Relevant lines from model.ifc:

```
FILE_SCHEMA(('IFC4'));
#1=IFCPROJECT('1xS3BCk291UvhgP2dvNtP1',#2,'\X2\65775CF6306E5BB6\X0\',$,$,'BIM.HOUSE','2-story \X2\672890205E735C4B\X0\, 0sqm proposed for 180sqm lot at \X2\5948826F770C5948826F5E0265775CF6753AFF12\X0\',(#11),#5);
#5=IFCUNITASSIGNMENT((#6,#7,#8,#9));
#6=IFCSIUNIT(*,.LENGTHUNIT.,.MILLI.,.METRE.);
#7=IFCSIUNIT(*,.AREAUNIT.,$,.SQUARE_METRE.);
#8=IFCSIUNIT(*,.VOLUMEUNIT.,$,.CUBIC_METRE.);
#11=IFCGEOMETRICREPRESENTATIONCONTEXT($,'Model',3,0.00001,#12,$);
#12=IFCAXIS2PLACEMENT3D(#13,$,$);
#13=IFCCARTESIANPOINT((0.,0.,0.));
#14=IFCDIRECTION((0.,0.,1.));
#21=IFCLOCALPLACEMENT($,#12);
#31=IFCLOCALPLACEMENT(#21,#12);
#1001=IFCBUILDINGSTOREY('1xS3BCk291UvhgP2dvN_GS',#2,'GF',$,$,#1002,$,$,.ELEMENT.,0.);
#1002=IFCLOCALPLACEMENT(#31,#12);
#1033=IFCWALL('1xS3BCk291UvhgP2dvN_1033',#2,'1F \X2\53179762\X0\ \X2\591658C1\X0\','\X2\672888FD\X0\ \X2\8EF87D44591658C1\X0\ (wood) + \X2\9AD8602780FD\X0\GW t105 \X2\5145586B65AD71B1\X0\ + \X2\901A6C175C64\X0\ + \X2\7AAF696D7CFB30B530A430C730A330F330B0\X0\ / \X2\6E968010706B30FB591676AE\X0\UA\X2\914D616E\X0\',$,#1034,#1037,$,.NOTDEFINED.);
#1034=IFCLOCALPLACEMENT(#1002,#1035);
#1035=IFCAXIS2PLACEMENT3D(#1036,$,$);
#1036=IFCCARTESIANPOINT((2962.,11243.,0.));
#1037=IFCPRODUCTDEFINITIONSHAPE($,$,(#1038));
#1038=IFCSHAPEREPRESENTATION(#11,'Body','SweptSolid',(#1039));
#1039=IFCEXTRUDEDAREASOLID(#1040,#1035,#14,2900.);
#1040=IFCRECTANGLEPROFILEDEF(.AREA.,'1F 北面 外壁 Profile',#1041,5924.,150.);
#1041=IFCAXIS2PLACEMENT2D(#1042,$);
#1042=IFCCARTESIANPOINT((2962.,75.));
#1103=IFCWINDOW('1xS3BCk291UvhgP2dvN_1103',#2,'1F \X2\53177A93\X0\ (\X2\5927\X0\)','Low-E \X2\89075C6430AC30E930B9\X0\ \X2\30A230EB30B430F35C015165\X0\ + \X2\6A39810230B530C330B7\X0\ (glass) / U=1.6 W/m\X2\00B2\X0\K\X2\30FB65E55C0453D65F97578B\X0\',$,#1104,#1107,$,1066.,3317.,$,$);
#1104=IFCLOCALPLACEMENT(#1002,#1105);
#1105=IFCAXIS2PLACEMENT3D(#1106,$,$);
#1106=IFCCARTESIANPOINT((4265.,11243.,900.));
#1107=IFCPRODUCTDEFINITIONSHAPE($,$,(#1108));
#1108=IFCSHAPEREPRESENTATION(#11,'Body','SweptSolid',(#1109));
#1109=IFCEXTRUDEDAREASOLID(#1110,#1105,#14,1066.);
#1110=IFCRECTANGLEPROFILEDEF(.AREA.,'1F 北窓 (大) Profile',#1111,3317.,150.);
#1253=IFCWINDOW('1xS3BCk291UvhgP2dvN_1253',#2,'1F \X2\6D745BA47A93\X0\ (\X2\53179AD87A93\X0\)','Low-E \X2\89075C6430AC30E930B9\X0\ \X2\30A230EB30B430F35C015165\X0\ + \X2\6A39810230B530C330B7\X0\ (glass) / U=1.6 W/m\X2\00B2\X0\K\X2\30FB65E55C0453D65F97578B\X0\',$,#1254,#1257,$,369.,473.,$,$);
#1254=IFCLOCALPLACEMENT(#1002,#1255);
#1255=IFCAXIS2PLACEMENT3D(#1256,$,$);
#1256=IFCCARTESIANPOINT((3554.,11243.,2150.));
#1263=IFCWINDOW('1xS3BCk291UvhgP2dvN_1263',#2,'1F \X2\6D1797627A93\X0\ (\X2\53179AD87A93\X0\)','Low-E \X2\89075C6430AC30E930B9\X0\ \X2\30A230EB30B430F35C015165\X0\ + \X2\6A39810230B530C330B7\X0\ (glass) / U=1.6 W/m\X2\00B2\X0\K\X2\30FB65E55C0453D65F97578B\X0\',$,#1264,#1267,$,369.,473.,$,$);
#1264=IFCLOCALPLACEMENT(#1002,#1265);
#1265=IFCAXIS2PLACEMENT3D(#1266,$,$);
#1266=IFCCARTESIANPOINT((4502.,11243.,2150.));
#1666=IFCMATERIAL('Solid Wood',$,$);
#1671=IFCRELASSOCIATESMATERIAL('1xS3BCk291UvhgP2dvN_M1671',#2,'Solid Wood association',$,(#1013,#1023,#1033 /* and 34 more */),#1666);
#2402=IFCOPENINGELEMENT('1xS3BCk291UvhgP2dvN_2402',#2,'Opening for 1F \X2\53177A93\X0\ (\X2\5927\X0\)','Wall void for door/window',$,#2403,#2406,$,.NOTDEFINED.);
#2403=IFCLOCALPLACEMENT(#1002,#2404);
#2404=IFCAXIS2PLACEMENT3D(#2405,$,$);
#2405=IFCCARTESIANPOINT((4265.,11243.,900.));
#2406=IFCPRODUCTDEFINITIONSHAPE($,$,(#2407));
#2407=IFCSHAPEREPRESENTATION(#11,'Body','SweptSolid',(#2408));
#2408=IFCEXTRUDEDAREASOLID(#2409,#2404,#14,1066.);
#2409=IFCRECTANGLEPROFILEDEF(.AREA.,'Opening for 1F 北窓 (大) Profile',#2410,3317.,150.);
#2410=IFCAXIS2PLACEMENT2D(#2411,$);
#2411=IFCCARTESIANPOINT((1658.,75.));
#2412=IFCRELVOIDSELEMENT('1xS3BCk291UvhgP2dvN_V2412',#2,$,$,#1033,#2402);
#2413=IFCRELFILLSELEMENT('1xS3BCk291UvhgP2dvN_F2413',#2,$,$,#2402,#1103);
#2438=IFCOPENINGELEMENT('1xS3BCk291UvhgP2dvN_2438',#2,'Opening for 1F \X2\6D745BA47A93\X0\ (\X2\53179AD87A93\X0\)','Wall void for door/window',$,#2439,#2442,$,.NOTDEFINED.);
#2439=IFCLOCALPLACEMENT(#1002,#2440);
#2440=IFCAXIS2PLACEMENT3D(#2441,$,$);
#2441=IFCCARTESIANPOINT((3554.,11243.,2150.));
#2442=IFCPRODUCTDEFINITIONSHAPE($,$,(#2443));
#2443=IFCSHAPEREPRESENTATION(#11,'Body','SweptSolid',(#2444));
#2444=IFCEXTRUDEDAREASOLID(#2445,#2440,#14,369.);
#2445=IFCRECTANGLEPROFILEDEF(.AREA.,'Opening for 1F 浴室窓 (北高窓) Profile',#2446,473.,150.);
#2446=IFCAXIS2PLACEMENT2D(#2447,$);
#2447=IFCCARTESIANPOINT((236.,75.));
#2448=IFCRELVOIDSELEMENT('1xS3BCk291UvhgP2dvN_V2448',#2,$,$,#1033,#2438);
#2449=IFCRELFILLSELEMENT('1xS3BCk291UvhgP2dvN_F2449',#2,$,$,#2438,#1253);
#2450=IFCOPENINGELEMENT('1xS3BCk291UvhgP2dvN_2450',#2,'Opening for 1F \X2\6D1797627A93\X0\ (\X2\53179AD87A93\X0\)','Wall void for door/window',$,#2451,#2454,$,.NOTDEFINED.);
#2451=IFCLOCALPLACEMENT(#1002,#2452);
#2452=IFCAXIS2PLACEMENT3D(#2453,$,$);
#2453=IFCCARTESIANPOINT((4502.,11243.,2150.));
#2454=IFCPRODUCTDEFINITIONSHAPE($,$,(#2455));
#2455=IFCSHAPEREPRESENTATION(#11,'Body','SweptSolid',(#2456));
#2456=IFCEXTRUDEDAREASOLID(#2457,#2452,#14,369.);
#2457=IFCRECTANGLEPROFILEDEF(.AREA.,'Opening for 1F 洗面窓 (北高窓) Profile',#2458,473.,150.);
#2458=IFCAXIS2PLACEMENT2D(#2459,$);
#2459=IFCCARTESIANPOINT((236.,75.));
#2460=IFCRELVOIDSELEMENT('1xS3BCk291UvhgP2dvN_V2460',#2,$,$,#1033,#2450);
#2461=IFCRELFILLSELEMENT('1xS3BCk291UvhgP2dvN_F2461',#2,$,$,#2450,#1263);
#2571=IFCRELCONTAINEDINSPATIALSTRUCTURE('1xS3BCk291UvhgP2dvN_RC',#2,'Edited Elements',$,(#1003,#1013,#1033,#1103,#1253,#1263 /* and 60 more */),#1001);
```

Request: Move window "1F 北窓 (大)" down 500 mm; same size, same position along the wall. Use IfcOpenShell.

```python
import numpy as np
import ifcopenshell
import ifcopenshell.api.geometry
import ifcopenshell.util.placement
import ifcopenshell.util.unit

model = ifcopenshell.open("model.ifc")
unit_scale = ifcopenshell.util.unit.calculate_unit_scale(model)

window = model.by_id(1103)
opening = window.FillsVoids[0].RelatingOpeningElement
dz = -0.5 / unit_scale

shift = np.array([0.0, 0.0, dz])
# The window is not placed relative to its opening, so move both.
for product in (opening, window):
    matrix = ifcopenshell.util.placement.get_local_placement(product.ObjectPlacement)
    matrix[:3, 3] += shift
    ifcopenshell.api.geometry.edit_object_placement(model, product=product, matrix=matrix, is_si=False)

print(f"moved by {dz * unit_scale:+.3f} m")

model.write("model_v2.ifc")
```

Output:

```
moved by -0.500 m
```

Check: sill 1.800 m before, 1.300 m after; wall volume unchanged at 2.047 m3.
